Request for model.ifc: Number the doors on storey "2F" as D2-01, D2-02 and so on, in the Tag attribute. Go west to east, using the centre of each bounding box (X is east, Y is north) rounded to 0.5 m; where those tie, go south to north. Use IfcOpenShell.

First a look at what the model holds.

```python
import ifcopenshell
import ifcopenshell.util.element
import ifcopenshell.util.placement

model = ifcopenshell.open("model.ifc")
print(model.schema)
storey = next(s for s in model.by_type("IfcBuildingStorey") if s.Name == "2F")
doors = [e for e in ifcopenshell.util.element.get_decomposition(storey) if e.is_a("IfcDoor")]
for e in sorted(doors, key=lambda e: e.id()):
    origin = ifcopenshell.util.placement.get_local_placement(e.ObjectPlacement)[:3, 3]
    print(e.id(), e.Tag, e.Name, origin.round(2) + 0.0, sep=" | ")
```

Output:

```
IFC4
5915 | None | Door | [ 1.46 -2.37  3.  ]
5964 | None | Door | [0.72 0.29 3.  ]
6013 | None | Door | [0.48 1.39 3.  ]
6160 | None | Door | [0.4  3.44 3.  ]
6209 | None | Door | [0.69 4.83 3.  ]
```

```python
import ifcopenshell
import ifcopenshell.geom
import ifcopenshell.util.element
import ifcopenshell.util.shape

model = ifcopenshell.open("model.ifc")
settings = ifcopenshell.geom.settings()
settings.set("use-world-coords", True)


def centre(element):
    shape = ifcopenshell.geom.create_shape(settings, element)
    return ifcopenshell.util.shape.get_bbox_centroid(shape.geometry)


storey = next(s for s in model.by_type("IfcBuildingStorey") if s.Name == "2F")
doors = [e for e in ifcopenshell.util.element.get_decomposition(storey) if e.is_a("IfcDoor")]

# Insertion points can sit at a corner or the storey origin, so sort by the geometry (in metres).
centres = {e: centre(e) for e in doors}
doors.sort(key=lambda e: (round(centres[e][0] / 0.5), centres[e][1]))

for i, e in enumerate(doors, start=1):
    number = f"D2-{i:02d}"
    e.Tag = number
    print(e.id(), number)

model.write("model_v2.ifc")
```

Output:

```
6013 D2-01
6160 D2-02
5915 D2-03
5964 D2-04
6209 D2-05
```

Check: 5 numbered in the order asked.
